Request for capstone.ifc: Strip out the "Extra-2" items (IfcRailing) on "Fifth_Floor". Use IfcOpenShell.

First a look at what the model holds.

```python
import ifcopenshell
import ifcopenshell.util.element

model = ifcopenshell.open("capstone.ifc")
print(model.schema)
storey = next(s for s in model.by_type("IfcBuildingStorey") if s.Name == "Fifth_Floor")
railings = [e for e in ifcopenshell.util.element.get_decomposition(storey) if e.is_a("IfcRailing")]
seen = {}
for e in railings:
    element_type = ifcopenshell.util.element.get_type(e)
    name = element_type.Name if element_type not in (None, e) else None
    seen[name] = seen.get(name, 0) + 1
for name, count in sorted(seen.items(), key=str):
    print(count, "x", name)
```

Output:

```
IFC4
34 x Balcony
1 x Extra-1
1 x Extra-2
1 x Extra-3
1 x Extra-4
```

```python
import ifcopenshell
import ifcopenshell.api.root
import ifcopenshell.util.element

model = ifcopenshell.open("capstone.ifc")

storey = next(s for s in model.by_type("IfcBuildingStorey") if s.Name == "Fifth_Floor")
railings = [e for e in ifcopenshell.util.element.get_decomposition(storey) if e.is_a("IfcRailing")]
targets = [e for e in railings if (t := ifcopenshell.util.element.get_type(e)) not in (None, e) and t.Name == "Extra-2"]

for e in targets:
    ifcopenshell.api.root.remove_product(model, product=e)
print(len(targets), "removed")

model.write("capstone_updated.ifc")
```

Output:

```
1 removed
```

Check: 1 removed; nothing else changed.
